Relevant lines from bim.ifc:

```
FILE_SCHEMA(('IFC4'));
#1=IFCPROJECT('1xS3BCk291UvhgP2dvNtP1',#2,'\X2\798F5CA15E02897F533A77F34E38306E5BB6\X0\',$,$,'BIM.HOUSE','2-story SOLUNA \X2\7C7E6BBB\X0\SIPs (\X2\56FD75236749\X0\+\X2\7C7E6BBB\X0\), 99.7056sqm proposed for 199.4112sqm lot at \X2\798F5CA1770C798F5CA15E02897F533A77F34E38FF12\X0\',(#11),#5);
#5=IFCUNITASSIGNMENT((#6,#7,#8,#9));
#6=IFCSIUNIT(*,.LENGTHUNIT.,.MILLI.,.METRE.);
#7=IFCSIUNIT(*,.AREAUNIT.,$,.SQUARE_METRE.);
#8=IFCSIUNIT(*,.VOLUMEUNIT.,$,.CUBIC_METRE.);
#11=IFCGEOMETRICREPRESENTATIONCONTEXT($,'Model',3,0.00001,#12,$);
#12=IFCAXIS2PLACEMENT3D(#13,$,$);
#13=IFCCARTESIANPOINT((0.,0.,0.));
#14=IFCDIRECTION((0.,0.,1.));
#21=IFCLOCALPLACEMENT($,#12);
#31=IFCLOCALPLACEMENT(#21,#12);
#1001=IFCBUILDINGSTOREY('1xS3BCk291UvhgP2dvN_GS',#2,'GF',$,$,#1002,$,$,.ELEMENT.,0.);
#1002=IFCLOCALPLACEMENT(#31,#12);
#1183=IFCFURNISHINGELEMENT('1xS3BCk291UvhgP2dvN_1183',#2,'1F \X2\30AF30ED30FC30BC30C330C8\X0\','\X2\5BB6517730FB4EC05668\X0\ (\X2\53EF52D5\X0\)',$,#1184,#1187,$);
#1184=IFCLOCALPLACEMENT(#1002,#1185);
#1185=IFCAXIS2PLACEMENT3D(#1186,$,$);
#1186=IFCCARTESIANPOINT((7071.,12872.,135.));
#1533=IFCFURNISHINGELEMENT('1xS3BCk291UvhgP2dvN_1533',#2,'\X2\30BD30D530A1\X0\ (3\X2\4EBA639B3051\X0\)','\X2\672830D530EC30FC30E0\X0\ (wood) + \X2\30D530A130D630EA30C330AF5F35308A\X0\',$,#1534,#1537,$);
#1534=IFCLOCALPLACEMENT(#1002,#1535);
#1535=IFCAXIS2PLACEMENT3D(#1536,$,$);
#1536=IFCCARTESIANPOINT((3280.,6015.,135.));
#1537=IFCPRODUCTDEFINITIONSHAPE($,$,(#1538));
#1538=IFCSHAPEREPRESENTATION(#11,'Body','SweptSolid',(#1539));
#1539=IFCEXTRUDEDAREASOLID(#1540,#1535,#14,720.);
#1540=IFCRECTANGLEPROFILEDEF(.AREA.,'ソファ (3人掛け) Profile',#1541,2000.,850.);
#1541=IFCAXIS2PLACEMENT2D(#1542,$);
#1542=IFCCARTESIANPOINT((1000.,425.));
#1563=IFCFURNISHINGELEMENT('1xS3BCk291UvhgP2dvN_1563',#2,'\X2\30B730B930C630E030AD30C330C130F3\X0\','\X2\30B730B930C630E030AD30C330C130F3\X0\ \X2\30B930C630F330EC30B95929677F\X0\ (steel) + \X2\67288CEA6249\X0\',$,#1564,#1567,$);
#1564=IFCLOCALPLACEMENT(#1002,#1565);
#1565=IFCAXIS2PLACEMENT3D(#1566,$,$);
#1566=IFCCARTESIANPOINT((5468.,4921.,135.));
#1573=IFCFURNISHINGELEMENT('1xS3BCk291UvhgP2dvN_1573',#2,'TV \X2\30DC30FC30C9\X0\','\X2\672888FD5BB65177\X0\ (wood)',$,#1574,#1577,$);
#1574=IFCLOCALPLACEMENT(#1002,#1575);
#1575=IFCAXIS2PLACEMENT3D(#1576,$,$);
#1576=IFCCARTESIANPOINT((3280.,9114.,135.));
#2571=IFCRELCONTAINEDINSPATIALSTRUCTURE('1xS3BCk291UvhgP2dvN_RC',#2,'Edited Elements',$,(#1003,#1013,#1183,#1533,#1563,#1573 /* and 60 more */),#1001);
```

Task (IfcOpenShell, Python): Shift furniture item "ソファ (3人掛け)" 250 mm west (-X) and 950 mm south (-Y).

```python
import ifcopenshell
import ifcopenshell.api.geometry
import ifcopenshell.util.placement
import ifcopenshell.util.unit

model = ifcopenshell.open("bim.ifc")
unit_scale = ifcopenshell.util.unit.calculate_unit_scale(model)

item = model.by_guid("1xS3BCk291UvhgP2dvN_1533")
matrix = ifcopenshell.util.placement.get_local_placement(item.ObjectPlacement)
matrix[0, 3] -= 0.25 / unit_scale
matrix[1, 3] -= 0.95 / unit_scale
ifcopenshell.api.geometry.edit_object_placement(model, product=item, matrix=matrix, is_si=False)

print(ifcopenshell.util.placement.get_local_placement(item.ObjectPlacement).round(3) + 0.0)

model.write("bim-out.ifc")
```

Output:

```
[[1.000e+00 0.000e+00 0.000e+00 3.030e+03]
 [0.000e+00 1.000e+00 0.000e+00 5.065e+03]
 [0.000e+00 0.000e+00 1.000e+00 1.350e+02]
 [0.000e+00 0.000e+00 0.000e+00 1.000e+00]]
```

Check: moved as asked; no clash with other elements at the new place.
